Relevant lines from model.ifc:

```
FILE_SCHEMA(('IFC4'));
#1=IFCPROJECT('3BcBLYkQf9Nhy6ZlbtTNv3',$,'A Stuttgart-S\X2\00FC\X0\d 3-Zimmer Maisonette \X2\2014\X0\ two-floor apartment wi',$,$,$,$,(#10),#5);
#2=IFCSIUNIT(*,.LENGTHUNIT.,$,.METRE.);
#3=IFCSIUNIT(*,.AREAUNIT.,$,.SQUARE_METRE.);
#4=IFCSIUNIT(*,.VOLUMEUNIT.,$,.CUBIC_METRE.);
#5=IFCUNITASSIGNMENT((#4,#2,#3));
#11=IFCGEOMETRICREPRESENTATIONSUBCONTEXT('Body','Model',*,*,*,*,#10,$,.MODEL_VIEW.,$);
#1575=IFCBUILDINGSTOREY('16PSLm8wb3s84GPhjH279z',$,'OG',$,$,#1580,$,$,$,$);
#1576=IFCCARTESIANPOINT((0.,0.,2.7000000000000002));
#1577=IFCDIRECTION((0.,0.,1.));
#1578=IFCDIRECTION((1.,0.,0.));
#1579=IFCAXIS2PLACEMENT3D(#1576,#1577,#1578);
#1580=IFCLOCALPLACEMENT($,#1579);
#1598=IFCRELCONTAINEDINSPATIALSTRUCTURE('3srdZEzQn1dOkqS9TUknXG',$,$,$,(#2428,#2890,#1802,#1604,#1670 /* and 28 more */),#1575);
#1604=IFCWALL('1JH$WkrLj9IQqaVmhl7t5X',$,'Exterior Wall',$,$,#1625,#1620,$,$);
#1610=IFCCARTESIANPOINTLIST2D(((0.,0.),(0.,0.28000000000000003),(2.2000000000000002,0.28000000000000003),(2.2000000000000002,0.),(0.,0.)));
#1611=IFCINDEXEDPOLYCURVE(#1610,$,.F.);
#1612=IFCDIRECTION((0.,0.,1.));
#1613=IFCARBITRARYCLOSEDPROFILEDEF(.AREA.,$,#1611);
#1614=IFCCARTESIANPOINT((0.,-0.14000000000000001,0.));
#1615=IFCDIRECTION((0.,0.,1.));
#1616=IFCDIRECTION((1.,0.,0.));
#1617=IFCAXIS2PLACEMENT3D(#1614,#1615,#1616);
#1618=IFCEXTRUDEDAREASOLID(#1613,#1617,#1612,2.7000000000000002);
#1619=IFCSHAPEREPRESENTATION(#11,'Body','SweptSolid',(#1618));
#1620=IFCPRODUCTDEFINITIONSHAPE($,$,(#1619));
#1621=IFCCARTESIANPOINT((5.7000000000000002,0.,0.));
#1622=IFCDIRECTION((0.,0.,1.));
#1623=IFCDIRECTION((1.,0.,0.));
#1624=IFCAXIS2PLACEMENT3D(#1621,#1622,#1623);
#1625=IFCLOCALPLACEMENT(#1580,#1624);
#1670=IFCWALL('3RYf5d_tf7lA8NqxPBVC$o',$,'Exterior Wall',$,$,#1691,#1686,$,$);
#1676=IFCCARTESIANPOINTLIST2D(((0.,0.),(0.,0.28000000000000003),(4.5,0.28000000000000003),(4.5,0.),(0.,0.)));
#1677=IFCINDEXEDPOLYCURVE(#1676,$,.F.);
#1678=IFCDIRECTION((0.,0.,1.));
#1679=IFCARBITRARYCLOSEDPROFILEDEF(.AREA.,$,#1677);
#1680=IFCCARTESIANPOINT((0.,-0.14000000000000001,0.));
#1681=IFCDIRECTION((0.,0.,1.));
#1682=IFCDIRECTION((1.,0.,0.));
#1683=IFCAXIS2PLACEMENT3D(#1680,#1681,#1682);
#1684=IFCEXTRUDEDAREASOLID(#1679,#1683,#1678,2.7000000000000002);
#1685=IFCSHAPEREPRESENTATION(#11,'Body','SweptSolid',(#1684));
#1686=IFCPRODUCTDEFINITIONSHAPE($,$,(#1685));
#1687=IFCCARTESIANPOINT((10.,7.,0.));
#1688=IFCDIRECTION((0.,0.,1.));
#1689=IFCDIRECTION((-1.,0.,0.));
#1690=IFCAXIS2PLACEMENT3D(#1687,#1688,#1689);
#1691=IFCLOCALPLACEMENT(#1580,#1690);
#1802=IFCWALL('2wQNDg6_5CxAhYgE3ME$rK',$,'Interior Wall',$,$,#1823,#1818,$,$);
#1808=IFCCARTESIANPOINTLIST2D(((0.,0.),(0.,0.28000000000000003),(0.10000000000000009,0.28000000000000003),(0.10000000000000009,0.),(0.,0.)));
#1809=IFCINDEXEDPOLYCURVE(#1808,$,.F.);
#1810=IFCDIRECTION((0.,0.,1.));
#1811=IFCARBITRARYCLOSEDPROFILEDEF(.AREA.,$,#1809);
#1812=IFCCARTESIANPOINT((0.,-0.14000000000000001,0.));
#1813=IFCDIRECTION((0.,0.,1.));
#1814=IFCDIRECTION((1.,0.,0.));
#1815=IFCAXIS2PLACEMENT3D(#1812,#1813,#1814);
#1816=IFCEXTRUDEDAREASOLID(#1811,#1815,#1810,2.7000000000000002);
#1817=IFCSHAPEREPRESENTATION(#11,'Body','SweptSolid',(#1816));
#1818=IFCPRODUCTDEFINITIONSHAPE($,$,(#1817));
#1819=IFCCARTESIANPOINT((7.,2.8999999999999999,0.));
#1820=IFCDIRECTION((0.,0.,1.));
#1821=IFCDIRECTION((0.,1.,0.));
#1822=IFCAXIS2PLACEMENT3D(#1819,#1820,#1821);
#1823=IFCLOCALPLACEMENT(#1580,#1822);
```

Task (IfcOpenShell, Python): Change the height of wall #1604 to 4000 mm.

```python
import ifcopenshell
import ifcopenshell.geom
import ifcopenshell.util.representation
import ifcopenshell.util.shape

model = ifcopenshell.open("model.ifc")
settings = ifcopenshell.geom.settings()


def volume(element):
    """Net volume in cubic metres, openings subtracted."""
    shape = ifcopenshell.geom.create_shape(settings, element)
    return ifcopenshell.util.shape.get_volume(shape.geometry)


wall = model.by_guid("1JH$WkrLj9IQqaVmhl7t5X")
before = volume(wall)

body = ifcopenshell.util.representation.get_representation(wall, "Model", "Body")
solid = body.Items[0]
old_height = solid.Depth
solid.Depth = 4.0
after = volume(wall)

print(f"height {old_height:g} -> {solid.Depth:g}, volume {before:.3f} -> {after:.3f} m3")

model.write("model_v2.ifc")
```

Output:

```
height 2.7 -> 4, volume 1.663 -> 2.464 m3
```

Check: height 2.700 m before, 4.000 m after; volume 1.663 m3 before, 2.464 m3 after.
